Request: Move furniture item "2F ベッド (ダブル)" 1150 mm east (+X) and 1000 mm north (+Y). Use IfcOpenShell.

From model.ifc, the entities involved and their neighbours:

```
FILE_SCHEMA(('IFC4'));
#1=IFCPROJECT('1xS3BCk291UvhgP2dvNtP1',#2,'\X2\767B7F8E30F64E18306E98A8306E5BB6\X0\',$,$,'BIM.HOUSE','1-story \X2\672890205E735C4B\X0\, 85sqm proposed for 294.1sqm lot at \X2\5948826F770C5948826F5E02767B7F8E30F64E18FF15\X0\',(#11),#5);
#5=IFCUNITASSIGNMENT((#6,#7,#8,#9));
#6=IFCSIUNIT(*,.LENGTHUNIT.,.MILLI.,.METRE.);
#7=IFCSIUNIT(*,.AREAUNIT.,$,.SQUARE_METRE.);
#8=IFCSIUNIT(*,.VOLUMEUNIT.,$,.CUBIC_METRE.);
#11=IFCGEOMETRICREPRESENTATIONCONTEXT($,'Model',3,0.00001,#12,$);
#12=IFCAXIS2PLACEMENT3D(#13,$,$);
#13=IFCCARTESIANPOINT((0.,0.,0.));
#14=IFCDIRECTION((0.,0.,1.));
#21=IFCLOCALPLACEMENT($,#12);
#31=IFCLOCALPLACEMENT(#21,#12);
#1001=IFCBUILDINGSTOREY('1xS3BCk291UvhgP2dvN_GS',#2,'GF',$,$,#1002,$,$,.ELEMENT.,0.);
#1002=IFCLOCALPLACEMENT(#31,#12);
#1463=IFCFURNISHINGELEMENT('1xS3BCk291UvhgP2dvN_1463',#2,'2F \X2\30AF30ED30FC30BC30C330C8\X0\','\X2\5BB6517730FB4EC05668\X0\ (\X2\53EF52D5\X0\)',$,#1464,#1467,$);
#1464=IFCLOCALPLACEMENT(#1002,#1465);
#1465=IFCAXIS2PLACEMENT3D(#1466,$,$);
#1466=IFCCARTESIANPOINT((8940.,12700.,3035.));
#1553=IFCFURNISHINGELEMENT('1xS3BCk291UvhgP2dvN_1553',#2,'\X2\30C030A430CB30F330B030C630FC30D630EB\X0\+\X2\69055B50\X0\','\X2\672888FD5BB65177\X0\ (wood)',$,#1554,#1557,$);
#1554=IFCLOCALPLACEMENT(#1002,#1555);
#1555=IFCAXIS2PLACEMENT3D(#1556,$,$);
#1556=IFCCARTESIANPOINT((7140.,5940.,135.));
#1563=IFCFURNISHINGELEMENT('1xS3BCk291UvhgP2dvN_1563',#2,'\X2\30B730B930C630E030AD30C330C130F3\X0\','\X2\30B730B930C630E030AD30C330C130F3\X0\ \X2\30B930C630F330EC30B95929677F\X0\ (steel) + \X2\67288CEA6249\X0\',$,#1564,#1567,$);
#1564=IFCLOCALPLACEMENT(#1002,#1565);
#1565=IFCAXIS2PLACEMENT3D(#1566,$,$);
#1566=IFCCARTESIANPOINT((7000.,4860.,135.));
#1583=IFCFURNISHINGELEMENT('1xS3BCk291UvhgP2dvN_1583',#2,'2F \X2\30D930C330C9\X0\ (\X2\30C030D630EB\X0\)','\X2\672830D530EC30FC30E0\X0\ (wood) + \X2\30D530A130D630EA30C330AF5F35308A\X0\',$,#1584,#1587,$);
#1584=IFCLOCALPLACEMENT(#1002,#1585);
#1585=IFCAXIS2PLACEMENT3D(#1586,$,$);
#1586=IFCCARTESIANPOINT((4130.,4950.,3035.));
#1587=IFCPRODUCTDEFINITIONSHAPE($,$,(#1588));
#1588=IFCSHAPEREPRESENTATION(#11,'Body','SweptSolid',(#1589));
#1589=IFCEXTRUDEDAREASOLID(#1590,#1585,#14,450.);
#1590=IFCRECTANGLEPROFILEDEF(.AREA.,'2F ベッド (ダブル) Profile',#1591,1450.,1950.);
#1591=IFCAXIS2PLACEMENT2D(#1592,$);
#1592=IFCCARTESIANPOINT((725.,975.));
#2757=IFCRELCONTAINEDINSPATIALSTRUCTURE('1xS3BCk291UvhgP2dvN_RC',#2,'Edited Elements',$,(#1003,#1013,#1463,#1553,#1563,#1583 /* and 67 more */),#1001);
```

```python
import ifcopenshell
import ifcopenshell.api.geometry
import ifcopenshell.util.placement
import ifcopenshell.util.unit

model = ifcopenshell.open("model.ifc")
unit_scale = ifcopenshell.util.unit.calculate_unit_scale(model)

item = model.by_id(1583)
matrix = ifcopenshell.util.placement.get_local_placement(item.ObjectPlacement)
matrix[0, 3] += 1.15 / unit_scale
matrix[1, 3] += 1 / unit_scale
ifcopenshell.api.geometry.edit_object_placement(model, product=item, matrix=matrix, is_si=False)

print(ifcopenshell.util.placement.get_local_placement(item.ObjectPlacement).round(3) + 0.0)

model.write("model_rev.ifc")
```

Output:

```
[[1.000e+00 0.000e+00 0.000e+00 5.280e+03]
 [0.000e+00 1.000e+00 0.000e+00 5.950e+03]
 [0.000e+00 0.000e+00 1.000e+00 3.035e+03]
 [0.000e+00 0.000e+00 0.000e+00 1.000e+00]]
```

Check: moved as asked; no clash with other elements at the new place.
